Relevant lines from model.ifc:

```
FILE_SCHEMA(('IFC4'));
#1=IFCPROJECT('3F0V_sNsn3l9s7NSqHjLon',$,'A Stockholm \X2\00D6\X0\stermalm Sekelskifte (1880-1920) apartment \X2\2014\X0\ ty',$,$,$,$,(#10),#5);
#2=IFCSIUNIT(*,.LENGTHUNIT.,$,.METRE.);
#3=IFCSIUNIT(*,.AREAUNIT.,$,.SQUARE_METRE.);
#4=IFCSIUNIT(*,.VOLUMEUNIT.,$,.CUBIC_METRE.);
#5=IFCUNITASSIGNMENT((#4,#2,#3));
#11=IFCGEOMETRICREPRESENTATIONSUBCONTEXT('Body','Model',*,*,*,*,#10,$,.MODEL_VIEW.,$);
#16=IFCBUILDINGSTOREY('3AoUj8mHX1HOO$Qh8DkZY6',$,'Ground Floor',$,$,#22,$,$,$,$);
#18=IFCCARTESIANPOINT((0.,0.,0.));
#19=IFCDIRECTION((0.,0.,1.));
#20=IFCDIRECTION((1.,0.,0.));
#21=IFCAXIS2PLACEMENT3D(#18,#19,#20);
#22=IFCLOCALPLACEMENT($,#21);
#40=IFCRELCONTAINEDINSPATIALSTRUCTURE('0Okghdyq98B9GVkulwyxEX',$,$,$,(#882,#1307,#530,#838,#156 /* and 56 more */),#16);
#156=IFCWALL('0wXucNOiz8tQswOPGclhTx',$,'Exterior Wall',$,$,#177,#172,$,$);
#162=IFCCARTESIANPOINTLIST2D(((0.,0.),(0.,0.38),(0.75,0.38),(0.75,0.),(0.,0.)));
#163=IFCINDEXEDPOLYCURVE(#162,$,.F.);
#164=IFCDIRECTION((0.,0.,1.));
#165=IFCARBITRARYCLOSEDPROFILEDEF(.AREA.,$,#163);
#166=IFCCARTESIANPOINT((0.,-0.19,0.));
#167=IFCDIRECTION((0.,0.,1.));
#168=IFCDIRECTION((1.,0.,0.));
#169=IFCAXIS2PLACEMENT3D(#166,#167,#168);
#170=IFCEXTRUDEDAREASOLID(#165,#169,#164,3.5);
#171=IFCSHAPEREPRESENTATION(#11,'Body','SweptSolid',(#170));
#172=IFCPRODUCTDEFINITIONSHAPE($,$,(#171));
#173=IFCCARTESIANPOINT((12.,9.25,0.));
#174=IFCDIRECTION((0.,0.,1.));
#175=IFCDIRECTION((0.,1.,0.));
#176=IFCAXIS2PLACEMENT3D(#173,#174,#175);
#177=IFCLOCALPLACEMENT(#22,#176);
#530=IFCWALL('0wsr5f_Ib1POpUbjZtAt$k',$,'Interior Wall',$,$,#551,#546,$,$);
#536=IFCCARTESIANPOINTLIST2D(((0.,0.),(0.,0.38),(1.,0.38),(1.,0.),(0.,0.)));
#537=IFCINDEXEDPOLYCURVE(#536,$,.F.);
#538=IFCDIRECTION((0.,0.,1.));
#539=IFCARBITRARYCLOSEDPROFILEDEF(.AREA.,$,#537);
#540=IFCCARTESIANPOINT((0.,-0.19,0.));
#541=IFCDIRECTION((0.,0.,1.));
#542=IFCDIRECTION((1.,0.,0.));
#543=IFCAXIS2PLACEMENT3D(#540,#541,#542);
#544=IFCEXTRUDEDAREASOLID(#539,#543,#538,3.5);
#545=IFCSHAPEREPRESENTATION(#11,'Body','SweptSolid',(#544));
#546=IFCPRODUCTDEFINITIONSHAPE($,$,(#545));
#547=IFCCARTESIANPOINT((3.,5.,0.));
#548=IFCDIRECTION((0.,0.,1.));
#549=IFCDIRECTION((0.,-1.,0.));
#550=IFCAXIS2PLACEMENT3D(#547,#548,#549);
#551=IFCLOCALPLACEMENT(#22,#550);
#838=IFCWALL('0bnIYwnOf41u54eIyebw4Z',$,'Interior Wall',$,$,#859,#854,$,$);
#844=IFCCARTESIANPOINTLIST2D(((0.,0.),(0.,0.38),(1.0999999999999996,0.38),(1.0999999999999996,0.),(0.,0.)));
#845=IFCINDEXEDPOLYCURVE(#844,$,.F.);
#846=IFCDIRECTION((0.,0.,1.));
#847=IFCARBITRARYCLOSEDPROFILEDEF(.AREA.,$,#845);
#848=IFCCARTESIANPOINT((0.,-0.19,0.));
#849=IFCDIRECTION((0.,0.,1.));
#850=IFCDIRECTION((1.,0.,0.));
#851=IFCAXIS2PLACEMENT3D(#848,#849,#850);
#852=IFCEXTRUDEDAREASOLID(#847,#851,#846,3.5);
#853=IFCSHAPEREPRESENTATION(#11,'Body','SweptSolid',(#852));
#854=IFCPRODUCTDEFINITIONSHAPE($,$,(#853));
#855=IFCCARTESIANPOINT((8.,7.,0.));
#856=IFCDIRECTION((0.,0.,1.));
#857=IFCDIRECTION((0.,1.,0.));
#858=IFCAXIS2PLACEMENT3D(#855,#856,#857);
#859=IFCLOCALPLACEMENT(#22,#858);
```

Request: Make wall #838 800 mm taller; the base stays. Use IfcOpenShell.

```python
import ifcopenshell
import ifcopenshell.geom
import ifcopenshell.util.representation
import ifcopenshell.util.shape
import ifcopenshell.util.unit

model = ifcopenshell.open("model.ifc")
unit_scale = ifcopenshell.util.unit.calculate_unit_scale(model)
settings = ifcopenshell.geom.settings()


def volume(element):
    """Net volume in cubic metres, openings subtracted."""
    shape = ifcopenshell.geom.create_shape(settings, element)
    return ifcopenshell.util.shape.get_volume(shape.geometry)


wall = model.by_id(838)
before = volume(wall)

body = ifcopenshell.util.representation.get_representation(wall, "Model", "Body")
solid = body.Items[0]
old_height = solid.Depth
solid.Depth += 0.8 / unit_scale
after = volume(wall)

print(f"height {old_height:g} -> {solid.Depth:g}, volume {before:.3f} -> {after:.3f} m3")

model.write("model_v2.ifc")
```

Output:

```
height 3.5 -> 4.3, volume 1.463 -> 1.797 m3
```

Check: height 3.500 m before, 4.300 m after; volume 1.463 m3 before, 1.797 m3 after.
